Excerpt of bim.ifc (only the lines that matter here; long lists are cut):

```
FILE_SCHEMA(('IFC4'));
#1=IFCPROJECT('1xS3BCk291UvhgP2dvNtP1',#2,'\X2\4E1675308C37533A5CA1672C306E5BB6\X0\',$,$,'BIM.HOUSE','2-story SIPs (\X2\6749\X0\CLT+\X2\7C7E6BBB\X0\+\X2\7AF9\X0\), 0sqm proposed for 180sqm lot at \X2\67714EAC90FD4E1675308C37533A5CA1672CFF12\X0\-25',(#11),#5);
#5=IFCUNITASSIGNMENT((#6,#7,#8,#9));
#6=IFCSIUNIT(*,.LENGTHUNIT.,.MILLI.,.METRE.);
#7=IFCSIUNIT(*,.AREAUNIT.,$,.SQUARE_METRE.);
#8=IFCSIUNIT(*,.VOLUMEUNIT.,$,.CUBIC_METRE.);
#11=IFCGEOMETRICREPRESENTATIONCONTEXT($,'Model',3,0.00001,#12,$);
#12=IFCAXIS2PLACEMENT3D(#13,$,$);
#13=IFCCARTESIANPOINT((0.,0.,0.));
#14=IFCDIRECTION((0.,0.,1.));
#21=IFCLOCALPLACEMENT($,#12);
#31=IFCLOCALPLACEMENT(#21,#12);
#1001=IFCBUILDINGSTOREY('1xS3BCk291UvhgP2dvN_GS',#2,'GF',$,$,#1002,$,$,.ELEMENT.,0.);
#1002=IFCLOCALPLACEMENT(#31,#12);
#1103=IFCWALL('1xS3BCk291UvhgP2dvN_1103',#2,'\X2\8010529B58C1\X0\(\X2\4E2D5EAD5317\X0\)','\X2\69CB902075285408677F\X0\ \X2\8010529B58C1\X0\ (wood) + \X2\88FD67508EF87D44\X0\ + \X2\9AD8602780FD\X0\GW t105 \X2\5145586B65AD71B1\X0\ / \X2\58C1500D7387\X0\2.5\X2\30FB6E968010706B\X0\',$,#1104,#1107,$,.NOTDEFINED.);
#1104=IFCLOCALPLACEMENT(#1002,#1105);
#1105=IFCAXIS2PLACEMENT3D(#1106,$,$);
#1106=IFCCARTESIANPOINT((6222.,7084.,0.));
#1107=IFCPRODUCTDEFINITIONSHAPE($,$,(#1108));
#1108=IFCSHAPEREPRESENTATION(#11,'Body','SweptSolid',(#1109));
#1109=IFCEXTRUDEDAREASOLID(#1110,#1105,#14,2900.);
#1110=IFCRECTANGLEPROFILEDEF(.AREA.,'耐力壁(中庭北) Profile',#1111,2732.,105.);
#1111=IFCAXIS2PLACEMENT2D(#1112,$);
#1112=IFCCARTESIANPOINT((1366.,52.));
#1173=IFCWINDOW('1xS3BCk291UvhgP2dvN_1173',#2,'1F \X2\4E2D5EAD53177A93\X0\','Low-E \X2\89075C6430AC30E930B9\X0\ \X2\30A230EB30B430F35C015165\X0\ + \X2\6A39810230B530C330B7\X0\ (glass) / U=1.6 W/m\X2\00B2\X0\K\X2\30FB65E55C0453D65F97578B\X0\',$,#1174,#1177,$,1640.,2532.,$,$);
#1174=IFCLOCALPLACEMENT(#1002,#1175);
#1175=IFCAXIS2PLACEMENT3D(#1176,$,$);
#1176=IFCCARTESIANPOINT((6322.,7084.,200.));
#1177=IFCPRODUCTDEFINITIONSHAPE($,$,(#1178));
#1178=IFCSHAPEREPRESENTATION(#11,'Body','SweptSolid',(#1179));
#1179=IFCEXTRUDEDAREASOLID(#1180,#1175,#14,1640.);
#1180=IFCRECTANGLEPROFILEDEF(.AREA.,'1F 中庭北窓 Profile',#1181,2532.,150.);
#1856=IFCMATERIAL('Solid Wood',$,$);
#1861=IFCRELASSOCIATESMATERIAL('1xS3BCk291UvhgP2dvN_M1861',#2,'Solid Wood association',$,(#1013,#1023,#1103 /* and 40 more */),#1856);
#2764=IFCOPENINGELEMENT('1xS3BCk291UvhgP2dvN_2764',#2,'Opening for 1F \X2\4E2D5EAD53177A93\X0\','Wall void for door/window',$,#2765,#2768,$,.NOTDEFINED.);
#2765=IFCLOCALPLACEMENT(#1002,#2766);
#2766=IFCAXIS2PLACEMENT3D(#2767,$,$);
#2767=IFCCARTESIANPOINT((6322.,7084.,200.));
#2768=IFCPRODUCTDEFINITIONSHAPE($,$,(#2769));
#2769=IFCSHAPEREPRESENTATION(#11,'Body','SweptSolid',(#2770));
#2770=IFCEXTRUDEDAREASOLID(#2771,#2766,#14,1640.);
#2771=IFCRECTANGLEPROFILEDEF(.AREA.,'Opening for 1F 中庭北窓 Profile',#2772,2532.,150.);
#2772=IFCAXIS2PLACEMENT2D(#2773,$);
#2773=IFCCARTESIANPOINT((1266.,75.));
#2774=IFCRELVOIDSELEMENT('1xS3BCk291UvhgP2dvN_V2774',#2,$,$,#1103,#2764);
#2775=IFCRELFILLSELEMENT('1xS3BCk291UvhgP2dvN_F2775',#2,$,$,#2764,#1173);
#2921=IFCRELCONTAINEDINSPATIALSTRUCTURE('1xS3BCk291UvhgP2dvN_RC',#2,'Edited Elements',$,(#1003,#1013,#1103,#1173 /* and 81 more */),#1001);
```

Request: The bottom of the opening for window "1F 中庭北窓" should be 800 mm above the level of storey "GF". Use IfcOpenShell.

```python
import numpy as np
import ifcopenshell
import ifcopenshell.api.geometry
import ifcopenshell.geom
import ifcopenshell.util.element
import ifcopenshell.util.placement
import ifcopenshell.util.shape
import ifcopenshell.util.unit

model = ifcopenshell.open("bim.ifc")
unit_scale = ifcopenshell.util.unit.calculate_unit_scale(model)

window = model.by_id(1173)
opening = window.FillsVoids[0].RelatingOpeningElement
storey = ifcopenshell.util.element.get_container(window, ifc_class="IfcBuildingStorey")
level = ifcopenshell.util.placement.get_local_placement(storey.ObjectPlacement)[2, 3]

# The opening's origin need not be at the sill, so measure its lowest point.
shape = ifcopenshell.geom.create_shape(ifcopenshell.geom.settings(), opening)
bottom = ifcopenshell.util.shape.get_shape_bottom_elevation(shape, shape.geometry) / unit_scale
dz = level + 800.0 - bottom

shift = np.array([0.0, 0.0, dz])
# The window is not placed relative to its opening, so move both.
for product in (opening, window):
    matrix = ifcopenshell.util.placement.get_local_placement(product.ObjectPlacement)
    matrix[:3, 3] += shift
    ifcopenshell.api.geometry.edit_object_placement(model, product=product, matrix=matrix, is_si=False)

print(f"moved by {dz * unit_scale:+.3f} m")

model.write("bim_updated.ifc")
```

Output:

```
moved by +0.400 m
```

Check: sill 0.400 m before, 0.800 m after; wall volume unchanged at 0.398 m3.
